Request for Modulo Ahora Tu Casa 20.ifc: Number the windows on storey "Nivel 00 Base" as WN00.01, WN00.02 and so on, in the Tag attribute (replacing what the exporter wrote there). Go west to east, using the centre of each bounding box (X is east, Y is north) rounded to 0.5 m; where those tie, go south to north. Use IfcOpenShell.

First a look at what the model holds.

```python
import ifcopenshell
import ifcopenshell.util.element
import ifcopenshell.util.placement

model = ifcopenshell.open("Modulo Ahora Tu Casa 20.ifc")
print(model.schema)
storey = next(s for s in model.by_type("IfcBuildingStorey") if s.Name == "Nivel 00 Base")
windows = [e for e in ifcopenshell.util.element.get_decomposition(storey) if e.is_a("IfcWindow")]
for e in sorted(windows, key=lambda e: e.id()):
    origin = ifcopenshell.util.placement.get_local_placement(e.ObjectPlacement)[:3, 3]
    print(e.id(), e.Tag, e.Name, origin.round(2) + 0.0, sep=" | ")
```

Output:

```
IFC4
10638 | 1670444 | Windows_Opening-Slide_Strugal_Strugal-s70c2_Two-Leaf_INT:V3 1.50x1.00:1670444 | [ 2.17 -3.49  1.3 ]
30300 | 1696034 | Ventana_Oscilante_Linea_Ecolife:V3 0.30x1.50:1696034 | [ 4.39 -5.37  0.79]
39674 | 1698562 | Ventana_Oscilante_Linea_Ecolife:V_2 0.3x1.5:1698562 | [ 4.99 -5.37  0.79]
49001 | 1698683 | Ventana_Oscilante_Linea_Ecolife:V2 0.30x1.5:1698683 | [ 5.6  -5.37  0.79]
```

```python
import ifcopenshell
import ifcopenshell.geom
import ifcopenshell.util.element
import ifcopenshell.util.shape

model = ifcopenshell.open("Modulo Ahora Tu Casa 20.ifc")
settings = ifcopenshell.geom.settings()
settings.set("use-world-coords", True)


def centre(element):
    shape = ifcopenshell.geom.create_shape(settings, element)
    return ifcopenshell.util.shape.get_bbox_centroid(shape.geometry)


storey = next(s for s in model.by_type("IfcBuildingStorey") if s.Name == "Nivel 00 Base")
windows = [e for e in ifcopenshell.util.element.get_decomposition(storey) if e.is_a("IfcWindow")]

# Insertion points can sit at a corner or the storey origin, so sort by the geometry (in metres).
centres = {e: centre(e) for e in windows}
windows.sort(key=lambda e: (round(centres[e][0] / 0.5), centres[e][1]))

for i, e in enumerate(windows, start=1):
    number = f"WN00.{i:02d}"
    e.Tag = number
    print(e.id(), number)

model.write("Modulo Ahora Tu Casa 20_rev.ifc")
```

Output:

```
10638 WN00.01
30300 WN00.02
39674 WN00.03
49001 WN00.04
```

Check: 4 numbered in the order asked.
